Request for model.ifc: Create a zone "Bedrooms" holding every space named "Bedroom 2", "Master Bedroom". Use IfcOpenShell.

First a look at what the model holds.

```python
import ifcopenshell

model = ifcopenshell.open("model.ifc")
print(model.schema)
seen = {}
for space in model.by_type("IfcSpace"):
    seen[space.LongName] = seen.get(space.LongName, 0) + 1
for name, count in sorted(seen.items(), key=str):
    print(count, "x", name)
print("zones:", [z.Name for z in model.by_type("IfcZone")][:20])
```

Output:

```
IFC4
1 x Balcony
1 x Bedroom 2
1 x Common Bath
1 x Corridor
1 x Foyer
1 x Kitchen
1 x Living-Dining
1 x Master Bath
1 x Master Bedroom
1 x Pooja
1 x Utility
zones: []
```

```python
import ifcopenshell
import ifcopenshell.api.group
import ifcopenshell.api.root

model = ifcopenshell.open("model.ifc")

names = {"Bedroom 2", "Master Bedroom"}
spaces = [s for s in model.by_type("IfcSpace") if s.LongName in names]

zone = ifcopenshell.api.root.create_entity(model, ifc_class="IfcZone", name="Bedrooms")
ifcopenshell.api.group.assign_group(model, products=spaces, group=zone)
print(len(spaces), "spaces in", zone.Name)

model.write("model-out.ifc")
```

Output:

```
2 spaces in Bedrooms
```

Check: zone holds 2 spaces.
